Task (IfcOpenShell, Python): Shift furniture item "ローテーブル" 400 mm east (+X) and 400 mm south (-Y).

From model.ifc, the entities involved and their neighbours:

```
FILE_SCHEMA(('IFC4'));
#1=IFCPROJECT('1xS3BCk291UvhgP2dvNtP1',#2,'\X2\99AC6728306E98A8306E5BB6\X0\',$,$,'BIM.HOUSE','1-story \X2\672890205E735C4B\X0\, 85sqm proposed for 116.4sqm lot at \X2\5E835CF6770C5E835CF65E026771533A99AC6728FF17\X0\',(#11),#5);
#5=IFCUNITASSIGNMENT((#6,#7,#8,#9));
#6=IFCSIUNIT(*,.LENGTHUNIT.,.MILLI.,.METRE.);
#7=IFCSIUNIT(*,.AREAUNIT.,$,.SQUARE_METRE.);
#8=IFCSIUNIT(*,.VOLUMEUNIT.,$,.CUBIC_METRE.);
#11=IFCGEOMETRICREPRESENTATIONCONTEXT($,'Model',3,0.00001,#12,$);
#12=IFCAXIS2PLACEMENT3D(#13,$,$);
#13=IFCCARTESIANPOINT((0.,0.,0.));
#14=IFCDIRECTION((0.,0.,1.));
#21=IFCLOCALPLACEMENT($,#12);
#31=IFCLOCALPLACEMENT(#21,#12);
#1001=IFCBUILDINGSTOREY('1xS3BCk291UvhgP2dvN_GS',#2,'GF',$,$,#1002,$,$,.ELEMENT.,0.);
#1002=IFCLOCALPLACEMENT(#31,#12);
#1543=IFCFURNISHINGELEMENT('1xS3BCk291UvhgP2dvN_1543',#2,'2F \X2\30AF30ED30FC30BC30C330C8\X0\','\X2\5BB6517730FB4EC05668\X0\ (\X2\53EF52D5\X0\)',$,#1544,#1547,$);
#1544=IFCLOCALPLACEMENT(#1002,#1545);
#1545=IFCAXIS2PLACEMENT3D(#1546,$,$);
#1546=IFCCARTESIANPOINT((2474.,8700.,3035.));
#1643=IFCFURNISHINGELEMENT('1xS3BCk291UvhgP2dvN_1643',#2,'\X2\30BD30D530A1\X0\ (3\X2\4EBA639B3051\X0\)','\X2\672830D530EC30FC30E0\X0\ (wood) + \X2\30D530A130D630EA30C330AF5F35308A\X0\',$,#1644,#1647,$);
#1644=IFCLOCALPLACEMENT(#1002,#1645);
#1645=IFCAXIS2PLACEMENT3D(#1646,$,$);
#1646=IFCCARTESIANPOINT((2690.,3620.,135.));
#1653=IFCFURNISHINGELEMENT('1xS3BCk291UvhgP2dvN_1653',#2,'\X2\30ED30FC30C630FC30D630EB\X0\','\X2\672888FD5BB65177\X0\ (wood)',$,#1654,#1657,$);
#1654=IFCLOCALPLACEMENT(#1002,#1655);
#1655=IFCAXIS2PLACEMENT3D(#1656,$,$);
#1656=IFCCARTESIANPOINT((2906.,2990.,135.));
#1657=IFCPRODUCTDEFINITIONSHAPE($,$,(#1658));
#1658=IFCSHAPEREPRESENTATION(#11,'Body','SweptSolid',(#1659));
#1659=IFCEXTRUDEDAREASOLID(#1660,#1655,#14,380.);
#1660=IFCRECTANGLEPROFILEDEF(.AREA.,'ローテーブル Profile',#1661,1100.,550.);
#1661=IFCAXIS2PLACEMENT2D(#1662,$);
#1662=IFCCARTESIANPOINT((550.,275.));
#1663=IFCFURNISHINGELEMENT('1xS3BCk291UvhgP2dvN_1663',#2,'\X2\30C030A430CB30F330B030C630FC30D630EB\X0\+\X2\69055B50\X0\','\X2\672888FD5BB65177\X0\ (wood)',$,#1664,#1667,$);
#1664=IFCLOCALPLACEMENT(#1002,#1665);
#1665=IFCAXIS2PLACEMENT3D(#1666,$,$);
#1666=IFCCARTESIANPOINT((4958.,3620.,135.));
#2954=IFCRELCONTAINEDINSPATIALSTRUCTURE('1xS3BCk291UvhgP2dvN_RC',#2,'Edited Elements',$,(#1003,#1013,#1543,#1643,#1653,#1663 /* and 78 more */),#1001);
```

```python
import ifcopenshell
import ifcopenshell.api.geometry
import ifcopenshell.util.placement
import ifcopenshell.util.unit

model = ifcopenshell.open("model.ifc")
unit_scale = ifcopenshell.util.unit.calculate_unit_scale(model)

item = model.by_id(1653)
matrix = ifcopenshell.util.placement.get_local_placement(item.ObjectPlacement)
matrix[0, 3] += 0.4 / unit_scale
matrix[1, 3] -= 0.4 / unit_scale
ifcopenshell.api.geometry.edit_object_placement(model, product=item, matrix=matrix, is_si=False)

print(ifcopenshell.util.placement.get_local_placement(item.ObjectPlacement).round(3) + 0.0)

model.write("model_updated.ifc")
```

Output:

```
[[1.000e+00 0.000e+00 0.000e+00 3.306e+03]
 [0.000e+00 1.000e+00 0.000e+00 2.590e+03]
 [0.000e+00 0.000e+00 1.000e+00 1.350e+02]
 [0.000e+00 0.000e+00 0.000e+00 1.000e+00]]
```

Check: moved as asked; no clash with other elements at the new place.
